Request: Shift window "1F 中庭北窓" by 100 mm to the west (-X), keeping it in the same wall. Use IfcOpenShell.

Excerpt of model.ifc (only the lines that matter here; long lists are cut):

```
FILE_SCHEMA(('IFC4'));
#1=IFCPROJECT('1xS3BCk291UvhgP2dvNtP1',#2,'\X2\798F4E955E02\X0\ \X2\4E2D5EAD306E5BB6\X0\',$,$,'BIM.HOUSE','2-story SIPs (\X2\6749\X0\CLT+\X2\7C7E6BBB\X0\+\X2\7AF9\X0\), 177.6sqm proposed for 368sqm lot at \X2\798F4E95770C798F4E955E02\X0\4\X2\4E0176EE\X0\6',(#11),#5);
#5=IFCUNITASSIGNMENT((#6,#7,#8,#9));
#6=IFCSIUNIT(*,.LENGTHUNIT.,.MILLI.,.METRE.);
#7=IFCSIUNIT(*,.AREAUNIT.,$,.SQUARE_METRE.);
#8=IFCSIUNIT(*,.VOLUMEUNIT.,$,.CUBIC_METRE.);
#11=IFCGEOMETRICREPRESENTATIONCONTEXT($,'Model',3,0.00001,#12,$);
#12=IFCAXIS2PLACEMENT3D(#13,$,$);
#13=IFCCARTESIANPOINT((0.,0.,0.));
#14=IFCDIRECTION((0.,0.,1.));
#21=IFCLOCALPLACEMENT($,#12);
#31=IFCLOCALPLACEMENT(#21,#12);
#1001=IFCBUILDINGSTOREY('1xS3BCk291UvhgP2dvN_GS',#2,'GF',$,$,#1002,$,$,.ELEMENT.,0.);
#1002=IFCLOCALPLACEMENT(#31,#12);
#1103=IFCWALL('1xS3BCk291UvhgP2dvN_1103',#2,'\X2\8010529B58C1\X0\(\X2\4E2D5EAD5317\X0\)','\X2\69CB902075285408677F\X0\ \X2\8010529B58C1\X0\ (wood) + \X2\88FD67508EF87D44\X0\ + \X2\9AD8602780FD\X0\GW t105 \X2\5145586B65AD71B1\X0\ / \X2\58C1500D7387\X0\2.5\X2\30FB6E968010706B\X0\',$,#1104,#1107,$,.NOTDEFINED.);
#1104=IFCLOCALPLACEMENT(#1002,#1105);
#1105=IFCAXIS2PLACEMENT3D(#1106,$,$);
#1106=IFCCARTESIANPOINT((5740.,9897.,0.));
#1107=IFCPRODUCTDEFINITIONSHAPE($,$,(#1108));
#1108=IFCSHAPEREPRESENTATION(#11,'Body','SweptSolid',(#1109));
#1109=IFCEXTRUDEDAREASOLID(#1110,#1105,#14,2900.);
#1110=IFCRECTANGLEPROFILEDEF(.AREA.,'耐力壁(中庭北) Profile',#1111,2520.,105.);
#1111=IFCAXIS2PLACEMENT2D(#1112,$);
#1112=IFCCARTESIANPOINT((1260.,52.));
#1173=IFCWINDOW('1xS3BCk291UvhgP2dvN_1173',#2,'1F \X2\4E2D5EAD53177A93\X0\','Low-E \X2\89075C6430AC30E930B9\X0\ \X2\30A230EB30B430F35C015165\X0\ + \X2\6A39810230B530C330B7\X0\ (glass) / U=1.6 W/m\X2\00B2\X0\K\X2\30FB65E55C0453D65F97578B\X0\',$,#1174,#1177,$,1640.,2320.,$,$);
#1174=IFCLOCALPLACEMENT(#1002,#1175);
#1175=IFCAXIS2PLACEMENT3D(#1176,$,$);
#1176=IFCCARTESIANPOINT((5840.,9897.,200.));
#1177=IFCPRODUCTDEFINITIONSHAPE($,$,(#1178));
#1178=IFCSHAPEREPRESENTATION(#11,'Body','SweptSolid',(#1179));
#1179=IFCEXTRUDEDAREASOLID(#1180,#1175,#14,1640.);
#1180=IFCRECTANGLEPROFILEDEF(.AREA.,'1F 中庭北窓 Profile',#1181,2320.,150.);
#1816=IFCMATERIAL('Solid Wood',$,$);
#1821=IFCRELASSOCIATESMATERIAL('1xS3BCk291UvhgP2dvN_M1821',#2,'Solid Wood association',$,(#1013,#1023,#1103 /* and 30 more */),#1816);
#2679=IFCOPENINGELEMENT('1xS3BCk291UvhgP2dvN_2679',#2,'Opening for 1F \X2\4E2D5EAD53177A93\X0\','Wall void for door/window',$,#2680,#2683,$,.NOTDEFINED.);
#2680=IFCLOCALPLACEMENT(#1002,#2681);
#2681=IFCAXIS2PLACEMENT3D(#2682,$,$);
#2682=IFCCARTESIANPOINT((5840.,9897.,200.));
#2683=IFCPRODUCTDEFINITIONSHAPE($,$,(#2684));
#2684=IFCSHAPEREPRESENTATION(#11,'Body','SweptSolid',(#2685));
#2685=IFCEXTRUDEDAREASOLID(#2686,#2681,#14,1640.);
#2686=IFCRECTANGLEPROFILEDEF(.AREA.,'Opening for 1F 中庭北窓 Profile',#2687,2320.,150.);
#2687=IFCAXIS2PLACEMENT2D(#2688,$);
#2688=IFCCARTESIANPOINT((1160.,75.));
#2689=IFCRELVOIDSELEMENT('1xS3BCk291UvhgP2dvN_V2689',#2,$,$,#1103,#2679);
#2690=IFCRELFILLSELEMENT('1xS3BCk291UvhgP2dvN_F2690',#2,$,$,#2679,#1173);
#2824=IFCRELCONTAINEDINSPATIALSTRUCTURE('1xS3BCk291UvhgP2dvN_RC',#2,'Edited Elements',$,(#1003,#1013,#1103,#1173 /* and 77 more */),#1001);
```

```python
import ifcopenshell
import ifcopenshell.api.geometry
import ifcopenshell.util.placement
import ifcopenshell.util.unit

model = ifcopenshell.open("model.ifc")
unit_scale = ifcopenshell.util.unit.calculate_unit_scale(model)

window = model.by_guid("1xS3BCk291UvhgP2dvN_1173")
opening = window.FillsVoids[0].RelatingOpeningElement
wall = opening.VoidsElements[0].RelatingBuildingElement

wall_matrix = ifcopenshell.util.placement.get_local_placement(wall.ObjectPlacement)
shift = wall_matrix[:3, 0] * -0.1 / unit_scale
before = ifcopenshell.util.placement.get_local_placement(window.ObjectPlacement)[:3, 3].copy()

# The window is not placed relative to its opening, so move both.
for product in (opening, window):
    matrix = ifcopenshell.util.placement.get_local_placement(product.ObjectPlacement)
    matrix[:3, 3] += shift
    ifcopenshell.api.geometry.edit_object_placement(model, product=product, matrix=matrix, is_si=False)

after = ifcopenshell.util.placement.get_local_placement(window.ObjectPlacement)[:3, 3]
print("window moved by", (after - before).round(3) + 0.0)

model.write("model_edited.ifc")
```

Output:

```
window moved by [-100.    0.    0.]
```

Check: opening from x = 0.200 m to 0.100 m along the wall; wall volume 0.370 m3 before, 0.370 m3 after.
